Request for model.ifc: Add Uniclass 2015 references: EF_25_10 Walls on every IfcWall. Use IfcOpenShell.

First a look at what the model holds.

```python
import ifcopenshell

model = ifcopenshell.open("model.ifc")
print(model.schema)
print("classifications:", [c.Name for c in model.by_type("IfcClassification")])
for ifc_class in ("IfcDoor", "IfcRoof", "IfcStair", "IfcWall", "IfcWindow"):
    print(ifc_class, len(model.by_type(ifc_class)))
```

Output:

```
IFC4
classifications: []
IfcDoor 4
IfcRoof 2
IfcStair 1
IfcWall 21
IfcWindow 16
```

```python
import ifcopenshell
import ifcopenshell.api.classification

model = ifcopenshell.open("model.ifc")

system = ifcopenshell.api.classification.add_classification(model, classification="Uniclass 2015")

codes = {
    "IfcWall": ("EF_25_10", "Walls"),
}
for ifc_class, (code, name) in codes.items():
    products = model.by_type(ifc_class)
    ifcopenshell.api.classification.add_reference(
        model, products=products, classification=system, identification=code, name=name
    )
    print(code, len(products))

model.write("model_v2.ifc")
```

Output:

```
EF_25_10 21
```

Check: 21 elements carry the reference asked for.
